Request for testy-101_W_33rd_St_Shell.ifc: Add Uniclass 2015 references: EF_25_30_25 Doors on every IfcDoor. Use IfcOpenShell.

First a look at what the model holds.

```python
import ifcopenshell

model = ifcopenshell.open("testy-101_W_33rd_St_Shell.ifc")
print(model.schema)
print("classifications:", [c.Name for c in model.by_type("IfcClassification")])
for ifc_class in ("IfcDoor", "IfcRoof", "IfcStair", "IfcWall", "IfcWindow"):
    print(ifc_class, len(model.by_type(ifc_class)))
```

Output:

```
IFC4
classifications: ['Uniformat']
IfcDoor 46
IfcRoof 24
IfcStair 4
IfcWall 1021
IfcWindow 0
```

```python
import ifcopenshell
import ifcopenshell.api.classification

model = ifcopenshell.open("testy-101_W_33rd_St_Shell.ifc")

system = ifcopenshell.api.classification.add_classification(model, classification="Uniclass 2015")

codes = {
    "IfcDoor": ("EF_25_30_25", "Doors"),
}
for ifc_class, (code, name) in codes.items():
    products = model.by_type(ifc_class)
    ifcopenshell.api.classification.add_reference(
        model, products=products, classification=system, identification=code, name=name
    )
    print(code, len(products))

model.write("testy-101_W_33rd_St_Shell_v2.ifc")
```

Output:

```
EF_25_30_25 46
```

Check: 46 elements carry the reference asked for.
